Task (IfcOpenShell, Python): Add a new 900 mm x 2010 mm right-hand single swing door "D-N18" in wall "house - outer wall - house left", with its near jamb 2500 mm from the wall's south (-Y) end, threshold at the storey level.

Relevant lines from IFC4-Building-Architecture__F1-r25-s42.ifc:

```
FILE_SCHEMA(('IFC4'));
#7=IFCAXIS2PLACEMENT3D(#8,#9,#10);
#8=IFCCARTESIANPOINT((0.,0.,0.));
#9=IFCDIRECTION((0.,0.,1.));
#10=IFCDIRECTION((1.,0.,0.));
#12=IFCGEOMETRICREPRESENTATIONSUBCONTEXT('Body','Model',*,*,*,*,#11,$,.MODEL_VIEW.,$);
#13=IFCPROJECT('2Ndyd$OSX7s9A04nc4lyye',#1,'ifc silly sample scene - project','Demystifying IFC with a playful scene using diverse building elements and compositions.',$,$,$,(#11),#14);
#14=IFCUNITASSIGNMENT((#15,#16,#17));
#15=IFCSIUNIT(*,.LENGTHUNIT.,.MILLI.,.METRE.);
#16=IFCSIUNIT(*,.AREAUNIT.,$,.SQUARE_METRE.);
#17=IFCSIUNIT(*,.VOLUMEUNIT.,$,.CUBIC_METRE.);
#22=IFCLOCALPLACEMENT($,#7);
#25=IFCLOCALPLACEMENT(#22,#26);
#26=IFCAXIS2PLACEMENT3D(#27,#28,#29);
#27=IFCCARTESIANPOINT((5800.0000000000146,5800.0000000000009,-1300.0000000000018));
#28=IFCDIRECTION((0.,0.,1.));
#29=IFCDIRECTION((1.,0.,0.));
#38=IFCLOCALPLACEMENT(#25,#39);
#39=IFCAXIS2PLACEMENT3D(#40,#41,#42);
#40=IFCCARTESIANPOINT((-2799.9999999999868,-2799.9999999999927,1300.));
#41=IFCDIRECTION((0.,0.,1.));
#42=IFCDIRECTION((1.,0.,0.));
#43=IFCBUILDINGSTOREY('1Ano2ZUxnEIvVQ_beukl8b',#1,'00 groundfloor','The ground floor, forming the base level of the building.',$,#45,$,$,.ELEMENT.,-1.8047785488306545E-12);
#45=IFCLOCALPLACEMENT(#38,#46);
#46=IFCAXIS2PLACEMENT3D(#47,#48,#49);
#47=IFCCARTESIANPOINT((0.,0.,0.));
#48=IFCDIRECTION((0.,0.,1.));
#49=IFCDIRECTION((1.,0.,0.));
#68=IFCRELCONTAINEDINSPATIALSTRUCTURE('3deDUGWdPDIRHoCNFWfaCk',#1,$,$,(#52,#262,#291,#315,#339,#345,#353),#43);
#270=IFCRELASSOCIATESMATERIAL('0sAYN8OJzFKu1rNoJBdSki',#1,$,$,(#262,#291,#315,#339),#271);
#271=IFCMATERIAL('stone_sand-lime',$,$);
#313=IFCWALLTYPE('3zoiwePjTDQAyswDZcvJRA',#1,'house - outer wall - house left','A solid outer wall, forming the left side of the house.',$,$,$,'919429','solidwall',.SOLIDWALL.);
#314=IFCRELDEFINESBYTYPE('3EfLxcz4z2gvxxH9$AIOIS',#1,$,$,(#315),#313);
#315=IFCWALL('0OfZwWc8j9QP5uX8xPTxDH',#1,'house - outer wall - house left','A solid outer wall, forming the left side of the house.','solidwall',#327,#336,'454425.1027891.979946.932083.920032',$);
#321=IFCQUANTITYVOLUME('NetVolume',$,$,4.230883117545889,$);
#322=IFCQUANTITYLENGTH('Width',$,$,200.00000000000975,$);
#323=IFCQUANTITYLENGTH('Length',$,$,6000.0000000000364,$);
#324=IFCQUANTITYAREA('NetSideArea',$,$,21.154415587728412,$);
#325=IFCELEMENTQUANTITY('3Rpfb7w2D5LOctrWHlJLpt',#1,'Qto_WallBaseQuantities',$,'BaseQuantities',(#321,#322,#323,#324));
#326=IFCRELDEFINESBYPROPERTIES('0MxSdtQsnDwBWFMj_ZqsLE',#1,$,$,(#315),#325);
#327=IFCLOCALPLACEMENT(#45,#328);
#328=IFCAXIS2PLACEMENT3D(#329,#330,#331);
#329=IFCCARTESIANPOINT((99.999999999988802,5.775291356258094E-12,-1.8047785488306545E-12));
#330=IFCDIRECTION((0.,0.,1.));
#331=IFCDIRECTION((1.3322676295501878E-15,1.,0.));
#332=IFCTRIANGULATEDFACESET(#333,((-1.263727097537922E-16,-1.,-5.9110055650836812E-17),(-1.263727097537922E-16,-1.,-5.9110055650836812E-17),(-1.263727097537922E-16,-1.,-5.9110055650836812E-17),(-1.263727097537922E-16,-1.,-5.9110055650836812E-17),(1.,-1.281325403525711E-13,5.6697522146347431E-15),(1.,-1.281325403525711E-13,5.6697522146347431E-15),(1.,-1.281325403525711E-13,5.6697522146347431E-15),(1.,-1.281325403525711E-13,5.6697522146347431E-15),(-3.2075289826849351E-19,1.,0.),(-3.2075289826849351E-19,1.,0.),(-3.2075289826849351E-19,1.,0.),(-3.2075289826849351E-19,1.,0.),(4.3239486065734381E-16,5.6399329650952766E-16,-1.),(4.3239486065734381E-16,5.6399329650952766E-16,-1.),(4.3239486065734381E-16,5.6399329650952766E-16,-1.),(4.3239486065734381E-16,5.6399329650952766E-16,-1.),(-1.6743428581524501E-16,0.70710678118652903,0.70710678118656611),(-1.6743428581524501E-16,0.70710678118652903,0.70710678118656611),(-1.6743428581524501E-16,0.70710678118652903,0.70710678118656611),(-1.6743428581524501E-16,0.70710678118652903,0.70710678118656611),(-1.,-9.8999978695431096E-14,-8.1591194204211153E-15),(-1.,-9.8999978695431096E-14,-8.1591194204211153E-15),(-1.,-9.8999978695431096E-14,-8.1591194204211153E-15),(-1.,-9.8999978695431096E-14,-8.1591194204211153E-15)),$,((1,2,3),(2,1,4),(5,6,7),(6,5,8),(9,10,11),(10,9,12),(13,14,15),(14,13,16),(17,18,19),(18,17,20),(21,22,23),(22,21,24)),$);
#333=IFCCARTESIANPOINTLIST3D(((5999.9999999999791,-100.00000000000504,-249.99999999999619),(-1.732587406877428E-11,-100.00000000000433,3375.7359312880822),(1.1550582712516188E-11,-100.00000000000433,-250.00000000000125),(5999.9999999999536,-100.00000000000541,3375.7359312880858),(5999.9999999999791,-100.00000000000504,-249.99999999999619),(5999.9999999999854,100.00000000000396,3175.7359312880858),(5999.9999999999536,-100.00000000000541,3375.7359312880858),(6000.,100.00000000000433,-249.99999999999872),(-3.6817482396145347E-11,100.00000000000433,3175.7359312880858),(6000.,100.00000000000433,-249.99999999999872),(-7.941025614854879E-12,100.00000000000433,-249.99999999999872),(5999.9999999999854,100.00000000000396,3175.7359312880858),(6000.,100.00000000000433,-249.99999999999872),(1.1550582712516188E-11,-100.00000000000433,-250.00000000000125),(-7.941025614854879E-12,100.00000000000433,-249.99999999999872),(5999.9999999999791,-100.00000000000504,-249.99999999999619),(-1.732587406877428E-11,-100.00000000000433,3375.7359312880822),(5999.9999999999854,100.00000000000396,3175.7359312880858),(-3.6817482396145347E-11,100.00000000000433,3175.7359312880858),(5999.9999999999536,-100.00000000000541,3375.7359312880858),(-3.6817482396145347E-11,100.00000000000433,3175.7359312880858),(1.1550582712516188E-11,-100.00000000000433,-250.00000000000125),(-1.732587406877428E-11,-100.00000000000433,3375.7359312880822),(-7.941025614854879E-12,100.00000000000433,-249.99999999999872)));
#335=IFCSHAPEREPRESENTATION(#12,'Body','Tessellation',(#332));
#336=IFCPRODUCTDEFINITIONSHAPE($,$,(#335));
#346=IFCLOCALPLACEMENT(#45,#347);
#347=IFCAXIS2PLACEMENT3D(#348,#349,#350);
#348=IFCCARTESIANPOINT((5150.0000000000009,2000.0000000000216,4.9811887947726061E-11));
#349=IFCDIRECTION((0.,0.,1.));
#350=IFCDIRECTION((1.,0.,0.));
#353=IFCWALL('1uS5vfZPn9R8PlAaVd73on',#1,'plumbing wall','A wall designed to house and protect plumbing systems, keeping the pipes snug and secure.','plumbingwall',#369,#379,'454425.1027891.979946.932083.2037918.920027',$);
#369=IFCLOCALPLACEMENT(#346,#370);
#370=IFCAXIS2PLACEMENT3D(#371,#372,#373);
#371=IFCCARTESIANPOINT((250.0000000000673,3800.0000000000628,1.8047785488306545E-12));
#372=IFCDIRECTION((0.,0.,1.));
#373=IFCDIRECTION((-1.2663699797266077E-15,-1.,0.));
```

```python
import numpy as np
import ifcopenshell
import ifcopenshell.api.feature
import ifcopenshell.api.geometry
import ifcopenshell.api.pset
import ifcopenshell.api.root
import ifcopenshell.api.spatial
import ifcopenshell.geom
import ifcopenshell.util.element
import ifcopenshell.util.placement
import ifcopenshell.util.representation
import ifcopenshell.util.shape
import ifcopenshell.util.unit

model = ifcopenshell.open("IFC4-Building-Architecture__F1-r25-s42.ifc")
unit_scale = ifcopenshell.util.unit.calculate_unit_scale(model)
area_scale = ifcopenshell.util.unit.calculate_unit_scale(model, "AREAUNIT")
volume_scale = ifcopenshell.util.unit.calculate_unit_scale(model, "VOLUMEUNIT")
settings = ifcopenshell.geom.settings()


def volume(element):
    """Net volume in cubic metres, openings subtracted."""
    shape = ifcopenshell.geom.create_shape(settings, element)
    return ifcopenshell.util.shape.get_volume(shape.geometry)


wall = model.by_guid("0OfZwWc8j9QP5uX8xPTxDH")
storey = ifcopenshell.util.element.get_container(wall, ifc_class="IfcBuildingStorey")
context = ifcopenshell.util.representation.get_context(model, "Model", "Body", "MODEL_VIEW")
before = volume(wall)

width, height, from_end, sill = 0.9, 2.01, 2.5, 0.0  # metres

# The wall runs along its own X axis, and the end named is its -X end.
wall_shape = ifcopenshell.geom.create_shape(settings, wall)
x, y, z = ifcopenshell.util.shape.get_vertices(wall_shape.geometry).T
start = x.min() + from_end
face, thickness = float(y.min()), float(y.max() - y.min())
wall_matrix = ifcopenshell.util.placement.get_local_placement(wall.ObjectPlacement)
level = ifcopenshell.util.placement.get_local_placement(storey.ObjectPlacement)[2, 3]


def in_wall(x, y):
    """Placement at x, y metres in the wall's axes, at sill height."""
    matrix = wall_matrix.copy()
    matrix[:, 3] = wall_matrix @ np.array([x / unit_scale, y / unit_scale, 0.0, 1.0])
    matrix[2, 3] = level + sill / unit_scale
    return matrix


# Opening: a box that overshoots both wall faces by 50 mm.
opening = ifcopenshell.api.root.create_entity(model, ifc_class="IfcOpeningElement", predefined_type="OPENING")
box = ifcopenshell.api.geometry.add_wall_representation(
    model, context=context, length=width, height=height, thickness=thickness + 0.1
)
ifcopenshell.api.geometry.assign_representation(model, product=opening, representation=box)
ifcopenshell.api.geometry.edit_object_placement(model, product=opening, matrix=in_wall(start, face - 0.05), is_si=False)
ifcopenshell.api.feature.add_feature(model, feature=opening, element=wall)

door = ifcopenshell.api.root.create_entity(model, ifc_class="IfcDoor", name="D-N18", predefined_type="DOOR")
door.OverallWidth, door.OverallHeight = width / unit_scale, height / unit_scale
door.OperationType = "SINGLE_SWING_RIGHT"
body = ifcopenshell.api.geometry.add_door_representation(
    model,
    context=context,
    overall_width=door.OverallWidth,
    overall_height=door.OverallHeight,
    operation_type="SINGLE_SWING_RIGHT",
    lining_properties={"LiningDepth": thickness / unit_scale, "ThresholdDepth": thickness / unit_scale},
)
ifcopenshell.api.geometry.assign_representation(model, product=door, representation=body)
ifcopenshell.api.spatial.assign_container(model, products=[door], relating_structure=storey)
ifcopenshell.api.feature.add_filling(model, opening=opening, element=door)

# The lining spans the wall, so the door starts at the wall face.
ifcopenshell.api.geometry.edit_object_placement(model, product=door, matrix=in_wall(start, face), is_si=False)

after = volume(wall)

# Update the wall's stored quantities.
qto = model.by_id(ifcopenshell.util.element.get_pset(wall, "Qto_WallBaseQuantities", should_inherit=False)["id"])
ifcopenshell.api.pset.edit_qto(model, qto=qto, properties={
    "NetVolume": after / volume_scale,
    "NetSideArea": after / thickness / area_scale,
})

print(f"wall volume {before:.3f} -> {after:.3f} m3")

model.write("IFC4-Building-Architecture__F1-r25-s42_edited.ifc")
```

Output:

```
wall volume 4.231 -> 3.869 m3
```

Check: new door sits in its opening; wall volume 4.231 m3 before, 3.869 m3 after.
